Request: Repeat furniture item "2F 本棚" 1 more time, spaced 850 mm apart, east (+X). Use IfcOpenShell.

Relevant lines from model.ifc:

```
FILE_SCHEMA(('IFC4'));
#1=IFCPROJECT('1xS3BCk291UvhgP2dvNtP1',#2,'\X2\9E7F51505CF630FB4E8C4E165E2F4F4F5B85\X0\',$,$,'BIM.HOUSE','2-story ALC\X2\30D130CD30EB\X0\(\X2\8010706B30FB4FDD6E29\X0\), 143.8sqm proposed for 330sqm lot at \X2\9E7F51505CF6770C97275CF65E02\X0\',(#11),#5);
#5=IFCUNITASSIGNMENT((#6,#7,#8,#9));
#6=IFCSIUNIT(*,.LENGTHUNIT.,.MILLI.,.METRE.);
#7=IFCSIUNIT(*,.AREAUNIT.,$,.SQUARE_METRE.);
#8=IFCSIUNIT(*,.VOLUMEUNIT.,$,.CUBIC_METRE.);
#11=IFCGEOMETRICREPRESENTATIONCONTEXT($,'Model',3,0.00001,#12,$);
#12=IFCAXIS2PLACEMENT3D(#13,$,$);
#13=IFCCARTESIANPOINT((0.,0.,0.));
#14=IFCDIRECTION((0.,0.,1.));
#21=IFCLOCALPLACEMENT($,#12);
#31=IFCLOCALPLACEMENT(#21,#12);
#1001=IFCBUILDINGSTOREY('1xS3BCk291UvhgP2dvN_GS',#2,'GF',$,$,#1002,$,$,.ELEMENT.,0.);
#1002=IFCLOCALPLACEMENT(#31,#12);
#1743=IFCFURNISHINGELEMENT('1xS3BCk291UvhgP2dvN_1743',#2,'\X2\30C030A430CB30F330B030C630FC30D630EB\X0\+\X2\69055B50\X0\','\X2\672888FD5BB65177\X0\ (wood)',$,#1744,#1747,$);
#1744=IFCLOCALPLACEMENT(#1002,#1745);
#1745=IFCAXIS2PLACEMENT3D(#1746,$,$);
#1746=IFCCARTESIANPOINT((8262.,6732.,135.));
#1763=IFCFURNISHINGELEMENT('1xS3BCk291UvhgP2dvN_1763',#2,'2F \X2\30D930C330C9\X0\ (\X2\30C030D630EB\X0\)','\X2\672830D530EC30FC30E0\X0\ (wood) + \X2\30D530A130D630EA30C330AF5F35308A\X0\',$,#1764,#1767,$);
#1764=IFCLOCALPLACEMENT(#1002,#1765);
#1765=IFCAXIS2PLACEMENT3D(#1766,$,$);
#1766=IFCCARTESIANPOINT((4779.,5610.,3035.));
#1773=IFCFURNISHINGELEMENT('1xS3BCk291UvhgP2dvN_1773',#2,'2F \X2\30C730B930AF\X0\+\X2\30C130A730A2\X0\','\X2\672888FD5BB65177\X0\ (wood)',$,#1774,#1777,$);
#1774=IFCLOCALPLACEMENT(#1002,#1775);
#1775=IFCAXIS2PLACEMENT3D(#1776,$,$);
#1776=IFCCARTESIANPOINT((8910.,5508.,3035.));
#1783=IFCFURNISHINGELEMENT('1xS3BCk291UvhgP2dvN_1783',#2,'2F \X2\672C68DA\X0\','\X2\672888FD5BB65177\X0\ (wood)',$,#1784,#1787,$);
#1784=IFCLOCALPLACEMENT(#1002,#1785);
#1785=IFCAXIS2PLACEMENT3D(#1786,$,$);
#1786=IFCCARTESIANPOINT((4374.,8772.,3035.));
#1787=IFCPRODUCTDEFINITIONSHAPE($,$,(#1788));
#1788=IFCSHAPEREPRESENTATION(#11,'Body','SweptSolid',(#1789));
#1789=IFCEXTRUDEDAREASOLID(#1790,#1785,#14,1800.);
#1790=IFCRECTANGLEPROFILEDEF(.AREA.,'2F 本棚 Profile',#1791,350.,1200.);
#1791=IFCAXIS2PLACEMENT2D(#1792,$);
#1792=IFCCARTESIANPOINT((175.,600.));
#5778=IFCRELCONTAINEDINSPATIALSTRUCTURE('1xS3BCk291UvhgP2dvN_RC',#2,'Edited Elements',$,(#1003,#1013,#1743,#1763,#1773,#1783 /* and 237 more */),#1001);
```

```python
import numpy as np
import ifcopenshell
import ifcopenshell.api.geometry
import ifcopenshell.api.root
import ifcopenshell.util.element
import ifcopenshell.util.placement

model = ifcopenshell.open("model.ifc")


def reuse_history(source, copy):
    """copy_class also copies each property set's owner history, people and application; keep the originals."""
    for rel in copy.IsDefinedBy:
        if rel.is_a("IfcRelDefinesByProperties") and (history := rel.RelatingPropertyDefinition.OwnerHistory):
            rel.RelatingPropertyDefinition.OwnerHistory = source.OwnerHistory
            ifcopenshell.util.element.remove_deep2(model, history)


source = model.by_guid("1xS3BCk291UvhgP2dvN_1783")
base = ifcopenshell.util.placement.get_local_placement(source.ObjectPlacement)
step = np.array([1.0, 0.0, 0.0]) * 850.0

for i in range(1, 2):
    copy = ifcopenshell.api.root.copy_class(model, product=source)
    copy.Representation = ifcopenshell.util.element.copy_deep(
        model, source.Representation, exclude=["IfcGeometricRepresentationContext", "IfcRepresentationMap"]
    )
    reuse_history(source, copy)
    matrix = base.copy()
    matrix[:3, 3] += i * step
    print("added at", matrix[:3, 3].round(3) + 0.0)
    ifcopenshell.api.geometry.edit_object_placement(model, product=copy, matrix=matrix, is_si=False)

model.write("model_updated.ifc")
```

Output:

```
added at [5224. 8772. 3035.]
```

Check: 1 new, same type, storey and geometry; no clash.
